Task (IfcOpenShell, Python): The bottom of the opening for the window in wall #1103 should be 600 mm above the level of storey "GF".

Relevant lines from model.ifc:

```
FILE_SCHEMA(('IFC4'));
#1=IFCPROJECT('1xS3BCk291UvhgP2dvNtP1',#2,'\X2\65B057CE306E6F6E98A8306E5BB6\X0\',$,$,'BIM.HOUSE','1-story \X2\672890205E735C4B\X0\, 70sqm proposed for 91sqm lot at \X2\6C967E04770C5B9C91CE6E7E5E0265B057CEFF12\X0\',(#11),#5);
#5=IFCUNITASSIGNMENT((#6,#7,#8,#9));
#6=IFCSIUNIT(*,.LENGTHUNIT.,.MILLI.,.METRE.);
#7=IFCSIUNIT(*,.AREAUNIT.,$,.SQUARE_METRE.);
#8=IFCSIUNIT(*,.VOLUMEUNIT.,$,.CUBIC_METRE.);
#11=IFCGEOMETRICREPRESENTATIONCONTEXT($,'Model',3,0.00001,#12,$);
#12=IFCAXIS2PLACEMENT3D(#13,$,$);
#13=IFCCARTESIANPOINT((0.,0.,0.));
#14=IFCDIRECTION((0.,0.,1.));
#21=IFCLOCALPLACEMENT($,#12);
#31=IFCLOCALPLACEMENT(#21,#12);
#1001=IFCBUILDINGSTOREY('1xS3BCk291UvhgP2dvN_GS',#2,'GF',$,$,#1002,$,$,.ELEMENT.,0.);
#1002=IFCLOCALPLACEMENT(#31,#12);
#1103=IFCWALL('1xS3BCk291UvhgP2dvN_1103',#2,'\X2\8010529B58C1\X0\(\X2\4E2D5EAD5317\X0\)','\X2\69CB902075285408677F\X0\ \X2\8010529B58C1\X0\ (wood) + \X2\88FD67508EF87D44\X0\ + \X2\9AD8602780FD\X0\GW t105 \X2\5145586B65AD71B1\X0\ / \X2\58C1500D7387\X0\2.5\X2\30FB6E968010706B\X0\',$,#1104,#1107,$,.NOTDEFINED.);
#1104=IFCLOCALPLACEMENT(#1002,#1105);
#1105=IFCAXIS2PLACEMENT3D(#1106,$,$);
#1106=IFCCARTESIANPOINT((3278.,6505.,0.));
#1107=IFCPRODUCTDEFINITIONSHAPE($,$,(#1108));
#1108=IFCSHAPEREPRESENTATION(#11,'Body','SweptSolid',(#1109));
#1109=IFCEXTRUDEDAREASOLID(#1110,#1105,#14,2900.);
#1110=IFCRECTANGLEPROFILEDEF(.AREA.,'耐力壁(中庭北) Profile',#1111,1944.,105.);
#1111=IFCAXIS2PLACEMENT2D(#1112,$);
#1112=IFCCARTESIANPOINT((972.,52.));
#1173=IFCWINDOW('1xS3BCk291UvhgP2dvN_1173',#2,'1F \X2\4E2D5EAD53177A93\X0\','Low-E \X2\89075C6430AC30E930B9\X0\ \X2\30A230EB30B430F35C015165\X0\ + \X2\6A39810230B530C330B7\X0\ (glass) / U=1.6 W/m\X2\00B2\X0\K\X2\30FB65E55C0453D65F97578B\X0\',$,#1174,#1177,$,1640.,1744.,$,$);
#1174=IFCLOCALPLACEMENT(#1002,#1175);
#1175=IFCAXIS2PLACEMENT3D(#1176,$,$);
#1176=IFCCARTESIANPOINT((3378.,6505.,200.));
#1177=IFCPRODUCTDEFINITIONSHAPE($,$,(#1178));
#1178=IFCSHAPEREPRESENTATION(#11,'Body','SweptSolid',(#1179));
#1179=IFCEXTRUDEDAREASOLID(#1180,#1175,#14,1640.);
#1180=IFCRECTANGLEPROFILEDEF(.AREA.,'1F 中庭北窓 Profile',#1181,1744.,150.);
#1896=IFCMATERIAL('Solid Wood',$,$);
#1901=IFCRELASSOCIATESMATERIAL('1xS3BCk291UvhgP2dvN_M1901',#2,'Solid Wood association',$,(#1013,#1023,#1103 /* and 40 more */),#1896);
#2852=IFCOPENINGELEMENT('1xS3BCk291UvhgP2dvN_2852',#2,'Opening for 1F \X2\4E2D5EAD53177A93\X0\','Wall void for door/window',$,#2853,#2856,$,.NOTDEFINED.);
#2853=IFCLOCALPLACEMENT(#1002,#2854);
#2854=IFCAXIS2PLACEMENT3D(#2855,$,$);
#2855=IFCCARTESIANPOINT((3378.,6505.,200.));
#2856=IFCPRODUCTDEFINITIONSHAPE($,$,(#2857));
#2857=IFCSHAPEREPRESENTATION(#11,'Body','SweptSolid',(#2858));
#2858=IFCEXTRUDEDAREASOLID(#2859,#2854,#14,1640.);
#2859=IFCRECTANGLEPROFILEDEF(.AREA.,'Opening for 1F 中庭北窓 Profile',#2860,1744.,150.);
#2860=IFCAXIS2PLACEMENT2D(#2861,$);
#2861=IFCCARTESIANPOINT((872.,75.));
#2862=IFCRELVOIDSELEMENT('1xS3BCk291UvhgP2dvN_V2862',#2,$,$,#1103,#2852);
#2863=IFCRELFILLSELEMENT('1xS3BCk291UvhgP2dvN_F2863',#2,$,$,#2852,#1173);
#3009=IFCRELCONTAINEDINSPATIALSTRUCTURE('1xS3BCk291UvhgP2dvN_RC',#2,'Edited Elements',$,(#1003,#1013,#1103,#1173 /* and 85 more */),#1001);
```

```python
import numpy as np
import ifcopenshell
import ifcopenshell.api.geometry
import ifcopenshell.geom
import ifcopenshell.util.element
import ifcopenshell.util.placement
import ifcopenshell.util.shape
import ifcopenshell.util.unit

model = ifcopenshell.open("model.ifc")
unit_scale = ifcopenshell.util.unit.calculate_unit_scale(model)

window = model.by_id(1173)
opening = window.FillsVoids[0].RelatingOpeningElement
storey = ifcopenshell.util.element.get_container(window, ifc_class="IfcBuildingStorey")
level = ifcopenshell.util.placement.get_local_placement(storey.ObjectPlacement)[2, 3]

# The opening's origin need not be at the sill, so measure its lowest point.
shape = ifcopenshell.geom.create_shape(ifcopenshell.geom.settings(), opening)
bottom = ifcopenshell.util.shape.get_shape_bottom_elevation(shape, shape.geometry) / unit_scale
dz = level + 0.6 / unit_scale - bottom

shift = np.array([0.0, 0.0, dz])
# The window is not placed relative to its opening, so move both.
for product in (opening, window):
    matrix = ifcopenshell.util.placement.get_local_placement(product.ObjectPlacement)
    matrix[:3, 3] += shift
    ifcopenshell.api.geometry.edit_object_placement(model, product=product, matrix=matrix, is_si=False)

print(f"moved by {dz * unit_scale:+.3f} m")

model.write("model_v2.ifc")
```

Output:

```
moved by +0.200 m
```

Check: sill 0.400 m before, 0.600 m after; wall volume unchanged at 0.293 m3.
